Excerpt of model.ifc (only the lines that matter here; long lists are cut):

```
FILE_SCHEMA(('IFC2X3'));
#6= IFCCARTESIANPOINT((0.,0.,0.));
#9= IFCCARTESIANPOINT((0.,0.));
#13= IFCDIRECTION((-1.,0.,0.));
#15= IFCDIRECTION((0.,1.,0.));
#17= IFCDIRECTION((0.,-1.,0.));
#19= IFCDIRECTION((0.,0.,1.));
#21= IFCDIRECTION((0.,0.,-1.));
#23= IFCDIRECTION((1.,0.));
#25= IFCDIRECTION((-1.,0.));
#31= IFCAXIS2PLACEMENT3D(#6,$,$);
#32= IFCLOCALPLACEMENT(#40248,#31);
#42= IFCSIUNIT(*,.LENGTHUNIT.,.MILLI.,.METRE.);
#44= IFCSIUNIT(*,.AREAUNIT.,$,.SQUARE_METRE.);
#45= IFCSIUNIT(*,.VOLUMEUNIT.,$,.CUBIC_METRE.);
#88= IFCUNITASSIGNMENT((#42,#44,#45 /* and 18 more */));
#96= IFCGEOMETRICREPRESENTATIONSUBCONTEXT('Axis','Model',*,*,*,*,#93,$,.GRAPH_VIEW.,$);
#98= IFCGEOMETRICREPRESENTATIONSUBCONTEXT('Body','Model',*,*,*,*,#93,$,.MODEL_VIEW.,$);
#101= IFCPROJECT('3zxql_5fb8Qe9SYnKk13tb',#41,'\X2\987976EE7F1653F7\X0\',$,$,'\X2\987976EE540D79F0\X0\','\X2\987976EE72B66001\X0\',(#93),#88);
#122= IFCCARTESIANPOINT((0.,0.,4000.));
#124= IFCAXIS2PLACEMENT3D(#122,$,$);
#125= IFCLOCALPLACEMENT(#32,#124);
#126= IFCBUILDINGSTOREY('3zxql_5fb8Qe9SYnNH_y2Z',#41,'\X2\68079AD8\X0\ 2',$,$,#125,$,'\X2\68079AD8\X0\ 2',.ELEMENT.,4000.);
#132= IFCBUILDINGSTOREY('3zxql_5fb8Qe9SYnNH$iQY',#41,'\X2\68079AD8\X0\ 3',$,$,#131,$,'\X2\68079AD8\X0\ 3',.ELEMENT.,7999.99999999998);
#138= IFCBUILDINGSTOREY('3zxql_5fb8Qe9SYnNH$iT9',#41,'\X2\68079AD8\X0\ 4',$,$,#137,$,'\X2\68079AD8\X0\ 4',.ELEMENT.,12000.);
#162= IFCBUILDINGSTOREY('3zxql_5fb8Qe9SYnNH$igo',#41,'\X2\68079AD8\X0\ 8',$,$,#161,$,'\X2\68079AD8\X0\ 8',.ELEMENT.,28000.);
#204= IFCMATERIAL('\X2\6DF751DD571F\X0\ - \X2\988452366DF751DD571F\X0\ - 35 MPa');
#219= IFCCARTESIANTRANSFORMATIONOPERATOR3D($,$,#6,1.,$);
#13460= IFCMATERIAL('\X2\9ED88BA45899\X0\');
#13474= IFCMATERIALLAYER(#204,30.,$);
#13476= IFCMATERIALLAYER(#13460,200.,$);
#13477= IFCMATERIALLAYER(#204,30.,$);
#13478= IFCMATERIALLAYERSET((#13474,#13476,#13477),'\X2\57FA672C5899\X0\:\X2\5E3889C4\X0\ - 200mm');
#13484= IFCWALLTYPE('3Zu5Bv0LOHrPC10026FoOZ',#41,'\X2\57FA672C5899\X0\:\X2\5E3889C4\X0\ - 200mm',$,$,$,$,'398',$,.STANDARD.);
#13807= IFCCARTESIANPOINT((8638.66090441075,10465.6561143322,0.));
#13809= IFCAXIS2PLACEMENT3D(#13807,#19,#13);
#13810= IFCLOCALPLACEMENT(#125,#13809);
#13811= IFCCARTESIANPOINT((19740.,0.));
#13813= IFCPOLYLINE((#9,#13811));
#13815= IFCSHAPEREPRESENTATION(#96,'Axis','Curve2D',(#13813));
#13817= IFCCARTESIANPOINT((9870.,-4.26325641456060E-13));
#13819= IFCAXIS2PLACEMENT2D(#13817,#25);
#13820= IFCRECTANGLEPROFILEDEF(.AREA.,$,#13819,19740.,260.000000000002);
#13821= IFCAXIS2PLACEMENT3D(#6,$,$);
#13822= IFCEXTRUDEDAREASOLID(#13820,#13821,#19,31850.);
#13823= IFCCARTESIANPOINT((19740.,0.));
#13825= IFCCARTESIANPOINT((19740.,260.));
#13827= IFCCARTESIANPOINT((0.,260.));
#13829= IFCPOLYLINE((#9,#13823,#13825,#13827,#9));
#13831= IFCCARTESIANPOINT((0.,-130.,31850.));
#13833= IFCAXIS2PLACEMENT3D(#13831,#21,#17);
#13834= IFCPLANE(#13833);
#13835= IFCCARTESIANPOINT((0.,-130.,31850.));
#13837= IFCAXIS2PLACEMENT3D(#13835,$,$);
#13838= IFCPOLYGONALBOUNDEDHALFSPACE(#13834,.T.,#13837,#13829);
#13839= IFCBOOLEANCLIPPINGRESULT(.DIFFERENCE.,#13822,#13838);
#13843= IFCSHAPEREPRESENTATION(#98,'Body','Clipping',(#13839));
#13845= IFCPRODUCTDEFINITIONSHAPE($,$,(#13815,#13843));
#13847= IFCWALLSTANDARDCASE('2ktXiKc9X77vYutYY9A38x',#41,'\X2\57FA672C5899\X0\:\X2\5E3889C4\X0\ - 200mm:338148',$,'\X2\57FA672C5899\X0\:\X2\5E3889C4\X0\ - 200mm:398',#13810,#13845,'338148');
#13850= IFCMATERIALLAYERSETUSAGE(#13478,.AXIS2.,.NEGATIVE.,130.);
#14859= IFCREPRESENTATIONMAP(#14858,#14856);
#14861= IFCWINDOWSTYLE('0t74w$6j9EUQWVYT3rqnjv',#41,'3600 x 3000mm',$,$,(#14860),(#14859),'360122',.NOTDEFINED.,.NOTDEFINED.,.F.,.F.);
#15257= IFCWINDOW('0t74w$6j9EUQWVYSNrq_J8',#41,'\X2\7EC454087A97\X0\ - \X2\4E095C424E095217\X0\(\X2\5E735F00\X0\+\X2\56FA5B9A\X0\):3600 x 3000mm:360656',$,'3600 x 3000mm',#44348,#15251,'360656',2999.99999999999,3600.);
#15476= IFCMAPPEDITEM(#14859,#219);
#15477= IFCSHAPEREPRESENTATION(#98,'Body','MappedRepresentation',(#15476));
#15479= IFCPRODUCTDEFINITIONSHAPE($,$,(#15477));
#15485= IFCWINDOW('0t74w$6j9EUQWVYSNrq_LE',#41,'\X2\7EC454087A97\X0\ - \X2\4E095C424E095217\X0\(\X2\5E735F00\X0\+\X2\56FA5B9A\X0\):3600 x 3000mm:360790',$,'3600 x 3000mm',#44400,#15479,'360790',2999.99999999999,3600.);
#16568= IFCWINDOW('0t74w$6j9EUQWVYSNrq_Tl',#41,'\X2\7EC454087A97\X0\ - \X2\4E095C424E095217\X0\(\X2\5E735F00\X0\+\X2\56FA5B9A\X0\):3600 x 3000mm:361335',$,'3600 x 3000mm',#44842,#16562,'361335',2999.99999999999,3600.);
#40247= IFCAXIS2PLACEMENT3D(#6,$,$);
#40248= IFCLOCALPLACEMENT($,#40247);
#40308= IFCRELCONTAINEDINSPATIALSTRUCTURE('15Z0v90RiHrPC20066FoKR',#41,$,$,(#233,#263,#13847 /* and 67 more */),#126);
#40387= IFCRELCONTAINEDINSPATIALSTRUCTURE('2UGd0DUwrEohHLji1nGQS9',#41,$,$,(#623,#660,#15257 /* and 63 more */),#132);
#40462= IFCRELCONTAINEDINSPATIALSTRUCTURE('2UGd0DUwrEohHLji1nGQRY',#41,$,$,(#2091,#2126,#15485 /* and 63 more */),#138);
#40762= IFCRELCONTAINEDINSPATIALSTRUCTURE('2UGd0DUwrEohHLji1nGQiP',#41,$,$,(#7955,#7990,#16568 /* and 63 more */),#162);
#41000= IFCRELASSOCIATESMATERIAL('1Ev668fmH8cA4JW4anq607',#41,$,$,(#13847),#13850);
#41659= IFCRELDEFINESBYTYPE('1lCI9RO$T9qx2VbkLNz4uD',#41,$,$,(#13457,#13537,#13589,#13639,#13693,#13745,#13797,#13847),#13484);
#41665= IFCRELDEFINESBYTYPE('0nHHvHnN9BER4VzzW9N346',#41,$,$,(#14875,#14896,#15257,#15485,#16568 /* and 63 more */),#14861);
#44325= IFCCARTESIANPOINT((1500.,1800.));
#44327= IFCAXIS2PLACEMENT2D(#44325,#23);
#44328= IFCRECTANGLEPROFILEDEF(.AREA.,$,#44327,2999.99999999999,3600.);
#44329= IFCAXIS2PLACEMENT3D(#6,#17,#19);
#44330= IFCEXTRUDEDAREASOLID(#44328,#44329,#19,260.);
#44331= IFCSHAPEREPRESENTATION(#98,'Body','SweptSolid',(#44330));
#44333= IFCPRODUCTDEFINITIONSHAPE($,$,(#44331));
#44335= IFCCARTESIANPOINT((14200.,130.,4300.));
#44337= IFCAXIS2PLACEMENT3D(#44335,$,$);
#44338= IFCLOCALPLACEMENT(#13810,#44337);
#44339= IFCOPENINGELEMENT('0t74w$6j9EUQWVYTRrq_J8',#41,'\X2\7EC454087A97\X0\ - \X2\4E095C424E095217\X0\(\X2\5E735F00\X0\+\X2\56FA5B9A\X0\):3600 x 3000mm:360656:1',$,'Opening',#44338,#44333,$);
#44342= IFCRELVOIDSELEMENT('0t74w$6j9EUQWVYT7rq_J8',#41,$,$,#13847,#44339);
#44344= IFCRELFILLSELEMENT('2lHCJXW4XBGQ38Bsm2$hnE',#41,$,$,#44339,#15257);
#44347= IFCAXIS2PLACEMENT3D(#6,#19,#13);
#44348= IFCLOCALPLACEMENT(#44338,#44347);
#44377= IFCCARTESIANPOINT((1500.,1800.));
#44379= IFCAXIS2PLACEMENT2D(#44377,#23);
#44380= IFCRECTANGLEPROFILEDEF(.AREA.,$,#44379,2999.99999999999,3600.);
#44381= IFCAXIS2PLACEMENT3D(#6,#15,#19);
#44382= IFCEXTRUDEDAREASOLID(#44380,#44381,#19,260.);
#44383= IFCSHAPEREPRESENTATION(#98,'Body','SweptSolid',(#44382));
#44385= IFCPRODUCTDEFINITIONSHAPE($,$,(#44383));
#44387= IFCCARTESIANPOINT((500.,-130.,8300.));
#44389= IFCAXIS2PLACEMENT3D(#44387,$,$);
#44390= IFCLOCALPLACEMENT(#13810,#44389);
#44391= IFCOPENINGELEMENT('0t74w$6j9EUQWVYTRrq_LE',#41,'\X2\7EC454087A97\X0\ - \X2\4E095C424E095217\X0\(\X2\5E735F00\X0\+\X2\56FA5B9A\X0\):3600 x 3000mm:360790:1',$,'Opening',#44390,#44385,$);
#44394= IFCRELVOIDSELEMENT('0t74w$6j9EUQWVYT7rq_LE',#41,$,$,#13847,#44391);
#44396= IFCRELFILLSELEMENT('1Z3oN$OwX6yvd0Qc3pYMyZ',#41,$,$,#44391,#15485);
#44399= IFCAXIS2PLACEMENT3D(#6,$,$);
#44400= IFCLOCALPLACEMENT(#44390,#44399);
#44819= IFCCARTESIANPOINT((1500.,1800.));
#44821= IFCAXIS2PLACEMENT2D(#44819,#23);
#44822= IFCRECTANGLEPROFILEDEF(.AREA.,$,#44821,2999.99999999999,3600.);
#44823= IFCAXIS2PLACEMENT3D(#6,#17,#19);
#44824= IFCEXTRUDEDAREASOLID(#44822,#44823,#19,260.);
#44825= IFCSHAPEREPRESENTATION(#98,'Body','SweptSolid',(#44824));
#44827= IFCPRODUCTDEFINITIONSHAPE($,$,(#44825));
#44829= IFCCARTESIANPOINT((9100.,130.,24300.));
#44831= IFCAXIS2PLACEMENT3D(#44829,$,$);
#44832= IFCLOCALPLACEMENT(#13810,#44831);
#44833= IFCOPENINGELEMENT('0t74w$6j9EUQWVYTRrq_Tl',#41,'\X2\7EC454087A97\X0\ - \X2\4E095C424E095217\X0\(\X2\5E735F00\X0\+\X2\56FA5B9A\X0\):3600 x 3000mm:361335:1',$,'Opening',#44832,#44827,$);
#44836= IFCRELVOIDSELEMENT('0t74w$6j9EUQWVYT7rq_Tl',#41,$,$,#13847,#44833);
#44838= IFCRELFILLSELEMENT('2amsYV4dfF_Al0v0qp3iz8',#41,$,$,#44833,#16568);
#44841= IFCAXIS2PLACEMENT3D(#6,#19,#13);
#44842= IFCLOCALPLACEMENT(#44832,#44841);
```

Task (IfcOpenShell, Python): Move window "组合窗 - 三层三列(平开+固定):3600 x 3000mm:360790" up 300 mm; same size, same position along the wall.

```python
import numpy as np
import ifcopenshell
import ifcopenshell.api.geometry
import ifcopenshell.util.placement
import ifcopenshell.util.unit

model = ifcopenshell.open("model.ifc")
unit_scale = ifcopenshell.util.unit.calculate_unit_scale(model)

window = model.by_guid("0t74w$6j9EUQWVYSNrq_LE")
opening = window.FillsVoids[0].RelatingOpeningElement
dz = 300.0

shift = np.array([0.0, 0.0, dz])
# The window is placed relative to its opening, so it follows when the opening moves.
matrix = ifcopenshell.util.placement.get_local_placement(opening.ObjectPlacement)
matrix[:3, 3] += shift
ifcopenshell.api.geometry.edit_object_placement(
    model, product=opening, matrix=matrix, is_si=False, should_transform_children=True
)

print(f"moved by {dz * unit_scale:+.3f} m")

model.write("model_edited.ifc")
```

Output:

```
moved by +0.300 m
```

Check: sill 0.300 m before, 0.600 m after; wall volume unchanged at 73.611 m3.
